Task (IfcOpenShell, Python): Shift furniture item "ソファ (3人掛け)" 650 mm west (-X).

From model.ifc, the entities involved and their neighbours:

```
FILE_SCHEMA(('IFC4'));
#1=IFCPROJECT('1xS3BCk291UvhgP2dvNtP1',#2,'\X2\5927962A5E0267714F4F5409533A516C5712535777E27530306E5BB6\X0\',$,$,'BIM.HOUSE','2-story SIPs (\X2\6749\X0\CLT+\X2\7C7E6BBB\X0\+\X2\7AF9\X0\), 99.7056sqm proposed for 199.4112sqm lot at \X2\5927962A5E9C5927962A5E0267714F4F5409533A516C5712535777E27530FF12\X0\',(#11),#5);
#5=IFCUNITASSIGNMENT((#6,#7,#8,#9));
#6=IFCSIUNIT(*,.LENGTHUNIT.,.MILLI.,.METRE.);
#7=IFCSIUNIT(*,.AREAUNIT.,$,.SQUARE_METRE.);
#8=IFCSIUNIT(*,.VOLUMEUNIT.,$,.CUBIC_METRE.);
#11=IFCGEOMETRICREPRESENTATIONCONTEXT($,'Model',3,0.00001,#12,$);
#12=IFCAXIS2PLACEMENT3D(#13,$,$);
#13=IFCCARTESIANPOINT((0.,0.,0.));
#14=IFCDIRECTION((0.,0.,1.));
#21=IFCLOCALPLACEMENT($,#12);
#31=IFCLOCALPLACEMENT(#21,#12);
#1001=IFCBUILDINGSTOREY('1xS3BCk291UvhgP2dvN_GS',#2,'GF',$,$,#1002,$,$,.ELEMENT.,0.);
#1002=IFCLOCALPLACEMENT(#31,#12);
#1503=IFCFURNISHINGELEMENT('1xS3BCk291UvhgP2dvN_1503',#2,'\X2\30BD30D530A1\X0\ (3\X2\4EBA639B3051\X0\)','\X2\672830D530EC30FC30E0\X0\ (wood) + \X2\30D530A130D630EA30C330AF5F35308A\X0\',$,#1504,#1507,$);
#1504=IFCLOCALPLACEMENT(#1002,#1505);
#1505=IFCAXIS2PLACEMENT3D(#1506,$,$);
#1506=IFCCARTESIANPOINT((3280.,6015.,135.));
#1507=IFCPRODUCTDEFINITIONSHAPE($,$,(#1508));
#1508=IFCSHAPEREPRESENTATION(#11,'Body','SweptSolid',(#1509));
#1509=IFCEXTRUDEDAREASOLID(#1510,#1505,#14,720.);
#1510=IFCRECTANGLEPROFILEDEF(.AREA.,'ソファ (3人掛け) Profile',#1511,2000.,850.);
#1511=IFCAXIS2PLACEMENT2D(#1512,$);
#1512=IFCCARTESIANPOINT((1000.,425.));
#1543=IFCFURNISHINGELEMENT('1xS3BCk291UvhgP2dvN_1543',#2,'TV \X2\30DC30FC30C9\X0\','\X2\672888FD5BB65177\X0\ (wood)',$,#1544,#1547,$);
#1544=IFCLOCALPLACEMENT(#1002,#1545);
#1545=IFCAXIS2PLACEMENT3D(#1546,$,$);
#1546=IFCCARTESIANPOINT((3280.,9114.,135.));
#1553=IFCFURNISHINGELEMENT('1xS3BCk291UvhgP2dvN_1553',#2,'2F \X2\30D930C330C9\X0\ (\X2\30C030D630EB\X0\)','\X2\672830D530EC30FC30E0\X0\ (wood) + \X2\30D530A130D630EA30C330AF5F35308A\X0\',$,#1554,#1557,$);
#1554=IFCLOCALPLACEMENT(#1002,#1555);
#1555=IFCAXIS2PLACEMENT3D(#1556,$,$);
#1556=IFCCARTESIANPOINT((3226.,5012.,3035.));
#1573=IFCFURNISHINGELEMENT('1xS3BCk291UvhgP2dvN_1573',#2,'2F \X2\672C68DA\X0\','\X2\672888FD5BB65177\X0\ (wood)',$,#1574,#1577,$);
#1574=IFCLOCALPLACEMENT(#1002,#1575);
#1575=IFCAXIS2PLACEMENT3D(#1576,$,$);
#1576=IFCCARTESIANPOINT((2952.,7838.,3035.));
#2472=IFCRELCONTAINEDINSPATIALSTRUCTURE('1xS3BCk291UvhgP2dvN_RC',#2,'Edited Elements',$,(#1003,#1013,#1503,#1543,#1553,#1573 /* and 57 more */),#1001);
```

```python
import ifcopenshell
import ifcopenshell.api.geometry
import ifcopenshell.util.placement
import ifcopenshell.util.unit

model = ifcopenshell.open("model.ifc")
unit_scale = ifcopenshell.util.unit.calculate_unit_scale(model)

item = model.by_guid("1xS3BCk291UvhgP2dvN_1503")
matrix = ifcopenshell.util.placement.get_local_placement(item.ObjectPlacement)
matrix[0, 3] -= 0.65 / unit_scale
ifcopenshell.api.geometry.edit_object_placement(model, product=item, matrix=matrix, is_si=False)

print(ifcopenshell.util.placement.get_local_placement(item.ObjectPlacement).round(3) + 0.0)

model.write("model_v2.ifc")
```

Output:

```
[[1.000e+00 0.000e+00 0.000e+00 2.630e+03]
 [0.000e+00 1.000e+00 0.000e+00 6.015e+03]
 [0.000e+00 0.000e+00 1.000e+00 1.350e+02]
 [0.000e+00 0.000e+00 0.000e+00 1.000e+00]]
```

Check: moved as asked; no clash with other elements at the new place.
